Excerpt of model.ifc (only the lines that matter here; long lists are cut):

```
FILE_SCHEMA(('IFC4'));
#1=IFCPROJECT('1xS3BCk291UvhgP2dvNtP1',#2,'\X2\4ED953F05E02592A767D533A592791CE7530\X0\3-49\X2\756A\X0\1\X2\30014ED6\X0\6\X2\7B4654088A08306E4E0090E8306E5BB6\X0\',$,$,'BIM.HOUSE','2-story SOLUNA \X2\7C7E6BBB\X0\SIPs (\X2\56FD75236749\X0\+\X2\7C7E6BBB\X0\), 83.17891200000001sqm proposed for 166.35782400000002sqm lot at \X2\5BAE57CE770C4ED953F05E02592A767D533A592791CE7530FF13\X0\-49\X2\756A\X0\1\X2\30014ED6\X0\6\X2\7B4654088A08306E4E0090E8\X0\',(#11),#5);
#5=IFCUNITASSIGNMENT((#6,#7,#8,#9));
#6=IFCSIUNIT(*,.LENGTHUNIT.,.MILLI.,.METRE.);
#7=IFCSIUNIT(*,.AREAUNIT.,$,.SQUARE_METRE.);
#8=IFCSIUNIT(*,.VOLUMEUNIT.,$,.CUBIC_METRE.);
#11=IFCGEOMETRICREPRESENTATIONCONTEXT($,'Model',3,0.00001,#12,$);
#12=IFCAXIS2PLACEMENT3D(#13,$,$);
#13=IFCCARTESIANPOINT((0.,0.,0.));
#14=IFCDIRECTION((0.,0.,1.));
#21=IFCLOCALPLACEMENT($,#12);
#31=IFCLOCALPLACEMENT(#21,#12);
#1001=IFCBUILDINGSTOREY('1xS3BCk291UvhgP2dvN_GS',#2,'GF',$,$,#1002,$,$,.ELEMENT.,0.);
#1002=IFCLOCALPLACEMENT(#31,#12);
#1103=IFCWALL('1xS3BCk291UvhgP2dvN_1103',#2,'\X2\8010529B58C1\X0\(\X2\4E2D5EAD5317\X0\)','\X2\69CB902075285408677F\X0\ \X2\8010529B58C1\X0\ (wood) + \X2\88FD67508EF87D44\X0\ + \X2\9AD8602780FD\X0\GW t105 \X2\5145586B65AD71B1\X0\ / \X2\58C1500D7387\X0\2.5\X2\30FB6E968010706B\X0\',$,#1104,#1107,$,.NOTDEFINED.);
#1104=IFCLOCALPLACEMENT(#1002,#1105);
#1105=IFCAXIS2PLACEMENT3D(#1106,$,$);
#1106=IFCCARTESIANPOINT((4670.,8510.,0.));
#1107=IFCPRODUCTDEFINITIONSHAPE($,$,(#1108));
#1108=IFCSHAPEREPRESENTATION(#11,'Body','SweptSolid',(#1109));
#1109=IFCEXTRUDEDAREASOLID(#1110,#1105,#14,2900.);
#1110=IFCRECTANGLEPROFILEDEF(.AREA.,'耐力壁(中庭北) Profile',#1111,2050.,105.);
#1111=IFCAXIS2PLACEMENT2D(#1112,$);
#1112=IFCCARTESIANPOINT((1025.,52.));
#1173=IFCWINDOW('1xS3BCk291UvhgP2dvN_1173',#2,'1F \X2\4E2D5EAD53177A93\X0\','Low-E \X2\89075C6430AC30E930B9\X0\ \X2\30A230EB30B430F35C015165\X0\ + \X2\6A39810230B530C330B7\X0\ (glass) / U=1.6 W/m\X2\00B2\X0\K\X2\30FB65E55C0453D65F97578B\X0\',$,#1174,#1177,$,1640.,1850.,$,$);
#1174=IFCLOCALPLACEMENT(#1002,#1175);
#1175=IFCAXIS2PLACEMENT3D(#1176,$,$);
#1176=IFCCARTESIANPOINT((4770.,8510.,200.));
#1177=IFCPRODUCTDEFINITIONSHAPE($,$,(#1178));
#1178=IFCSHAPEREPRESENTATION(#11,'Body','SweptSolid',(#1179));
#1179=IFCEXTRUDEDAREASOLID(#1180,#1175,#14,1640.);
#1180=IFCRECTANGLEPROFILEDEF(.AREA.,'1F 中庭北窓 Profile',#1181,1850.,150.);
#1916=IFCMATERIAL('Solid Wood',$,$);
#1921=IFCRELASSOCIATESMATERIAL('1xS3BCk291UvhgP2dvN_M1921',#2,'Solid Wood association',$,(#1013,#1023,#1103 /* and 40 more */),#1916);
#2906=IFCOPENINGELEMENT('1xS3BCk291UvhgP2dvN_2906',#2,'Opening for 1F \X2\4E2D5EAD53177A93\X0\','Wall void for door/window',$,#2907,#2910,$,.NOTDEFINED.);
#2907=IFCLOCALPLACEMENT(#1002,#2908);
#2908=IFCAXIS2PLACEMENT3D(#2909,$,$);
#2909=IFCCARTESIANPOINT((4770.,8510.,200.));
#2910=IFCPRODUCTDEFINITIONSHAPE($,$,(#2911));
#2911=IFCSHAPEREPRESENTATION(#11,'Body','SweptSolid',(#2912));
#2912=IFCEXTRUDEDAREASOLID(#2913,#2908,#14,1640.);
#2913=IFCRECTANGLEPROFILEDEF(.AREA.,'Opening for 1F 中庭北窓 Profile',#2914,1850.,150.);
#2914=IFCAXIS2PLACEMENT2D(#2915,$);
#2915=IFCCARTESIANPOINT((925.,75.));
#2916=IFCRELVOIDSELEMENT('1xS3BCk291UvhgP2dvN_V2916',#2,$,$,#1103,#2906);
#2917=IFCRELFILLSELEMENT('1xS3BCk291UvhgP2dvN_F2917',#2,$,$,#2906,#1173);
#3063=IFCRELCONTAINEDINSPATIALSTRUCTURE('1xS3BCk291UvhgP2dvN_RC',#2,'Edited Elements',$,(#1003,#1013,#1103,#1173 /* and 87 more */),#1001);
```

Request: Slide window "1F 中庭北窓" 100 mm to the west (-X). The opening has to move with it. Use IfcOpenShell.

```python
import ifcopenshell
import ifcopenshell.api.geometry
import ifcopenshell.util.placement
import ifcopenshell.util.unit

model = ifcopenshell.open("model.ifc")
unit_scale = ifcopenshell.util.unit.calculate_unit_scale(model)

window = model.by_guid("1xS3BCk291UvhgP2dvN_1173")
opening = window.FillsVoids[0].RelatingOpeningElement
wall = opening.VoidsElements[0].RelatingBuildingElement

wall_matrix = ifcopenshell.util.placement.get_local_placement(wall.ObjectPlacement)
shift = wall_matrix[:3, 0] * -0.1 / unit_scale
before = ifcopenshell.util.placement.get_local_placement(window.ObjectPlacement)[:3, 3].copy()

# The window is not placed relative to its opening, so move both.
for product in (opening, window):
    matrix = ifcopenshell.util.placement.get_local_placement(product.ObjectPlacement)
    matrix[:3, 3] += shift
    ifcopenshell.api.geometry.edit_object_placement(model, product=product, matrix=matrix, is_si=False)

after = ifcopenshell.util.placement.get_local_placement(window.ObjectPlacement)[:3, 3]
print("window moved by", (after - before).round(3) + 0.0)

model.write("model-out.ifc")
```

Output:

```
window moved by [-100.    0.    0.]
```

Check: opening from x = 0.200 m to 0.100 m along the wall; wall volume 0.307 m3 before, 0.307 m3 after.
